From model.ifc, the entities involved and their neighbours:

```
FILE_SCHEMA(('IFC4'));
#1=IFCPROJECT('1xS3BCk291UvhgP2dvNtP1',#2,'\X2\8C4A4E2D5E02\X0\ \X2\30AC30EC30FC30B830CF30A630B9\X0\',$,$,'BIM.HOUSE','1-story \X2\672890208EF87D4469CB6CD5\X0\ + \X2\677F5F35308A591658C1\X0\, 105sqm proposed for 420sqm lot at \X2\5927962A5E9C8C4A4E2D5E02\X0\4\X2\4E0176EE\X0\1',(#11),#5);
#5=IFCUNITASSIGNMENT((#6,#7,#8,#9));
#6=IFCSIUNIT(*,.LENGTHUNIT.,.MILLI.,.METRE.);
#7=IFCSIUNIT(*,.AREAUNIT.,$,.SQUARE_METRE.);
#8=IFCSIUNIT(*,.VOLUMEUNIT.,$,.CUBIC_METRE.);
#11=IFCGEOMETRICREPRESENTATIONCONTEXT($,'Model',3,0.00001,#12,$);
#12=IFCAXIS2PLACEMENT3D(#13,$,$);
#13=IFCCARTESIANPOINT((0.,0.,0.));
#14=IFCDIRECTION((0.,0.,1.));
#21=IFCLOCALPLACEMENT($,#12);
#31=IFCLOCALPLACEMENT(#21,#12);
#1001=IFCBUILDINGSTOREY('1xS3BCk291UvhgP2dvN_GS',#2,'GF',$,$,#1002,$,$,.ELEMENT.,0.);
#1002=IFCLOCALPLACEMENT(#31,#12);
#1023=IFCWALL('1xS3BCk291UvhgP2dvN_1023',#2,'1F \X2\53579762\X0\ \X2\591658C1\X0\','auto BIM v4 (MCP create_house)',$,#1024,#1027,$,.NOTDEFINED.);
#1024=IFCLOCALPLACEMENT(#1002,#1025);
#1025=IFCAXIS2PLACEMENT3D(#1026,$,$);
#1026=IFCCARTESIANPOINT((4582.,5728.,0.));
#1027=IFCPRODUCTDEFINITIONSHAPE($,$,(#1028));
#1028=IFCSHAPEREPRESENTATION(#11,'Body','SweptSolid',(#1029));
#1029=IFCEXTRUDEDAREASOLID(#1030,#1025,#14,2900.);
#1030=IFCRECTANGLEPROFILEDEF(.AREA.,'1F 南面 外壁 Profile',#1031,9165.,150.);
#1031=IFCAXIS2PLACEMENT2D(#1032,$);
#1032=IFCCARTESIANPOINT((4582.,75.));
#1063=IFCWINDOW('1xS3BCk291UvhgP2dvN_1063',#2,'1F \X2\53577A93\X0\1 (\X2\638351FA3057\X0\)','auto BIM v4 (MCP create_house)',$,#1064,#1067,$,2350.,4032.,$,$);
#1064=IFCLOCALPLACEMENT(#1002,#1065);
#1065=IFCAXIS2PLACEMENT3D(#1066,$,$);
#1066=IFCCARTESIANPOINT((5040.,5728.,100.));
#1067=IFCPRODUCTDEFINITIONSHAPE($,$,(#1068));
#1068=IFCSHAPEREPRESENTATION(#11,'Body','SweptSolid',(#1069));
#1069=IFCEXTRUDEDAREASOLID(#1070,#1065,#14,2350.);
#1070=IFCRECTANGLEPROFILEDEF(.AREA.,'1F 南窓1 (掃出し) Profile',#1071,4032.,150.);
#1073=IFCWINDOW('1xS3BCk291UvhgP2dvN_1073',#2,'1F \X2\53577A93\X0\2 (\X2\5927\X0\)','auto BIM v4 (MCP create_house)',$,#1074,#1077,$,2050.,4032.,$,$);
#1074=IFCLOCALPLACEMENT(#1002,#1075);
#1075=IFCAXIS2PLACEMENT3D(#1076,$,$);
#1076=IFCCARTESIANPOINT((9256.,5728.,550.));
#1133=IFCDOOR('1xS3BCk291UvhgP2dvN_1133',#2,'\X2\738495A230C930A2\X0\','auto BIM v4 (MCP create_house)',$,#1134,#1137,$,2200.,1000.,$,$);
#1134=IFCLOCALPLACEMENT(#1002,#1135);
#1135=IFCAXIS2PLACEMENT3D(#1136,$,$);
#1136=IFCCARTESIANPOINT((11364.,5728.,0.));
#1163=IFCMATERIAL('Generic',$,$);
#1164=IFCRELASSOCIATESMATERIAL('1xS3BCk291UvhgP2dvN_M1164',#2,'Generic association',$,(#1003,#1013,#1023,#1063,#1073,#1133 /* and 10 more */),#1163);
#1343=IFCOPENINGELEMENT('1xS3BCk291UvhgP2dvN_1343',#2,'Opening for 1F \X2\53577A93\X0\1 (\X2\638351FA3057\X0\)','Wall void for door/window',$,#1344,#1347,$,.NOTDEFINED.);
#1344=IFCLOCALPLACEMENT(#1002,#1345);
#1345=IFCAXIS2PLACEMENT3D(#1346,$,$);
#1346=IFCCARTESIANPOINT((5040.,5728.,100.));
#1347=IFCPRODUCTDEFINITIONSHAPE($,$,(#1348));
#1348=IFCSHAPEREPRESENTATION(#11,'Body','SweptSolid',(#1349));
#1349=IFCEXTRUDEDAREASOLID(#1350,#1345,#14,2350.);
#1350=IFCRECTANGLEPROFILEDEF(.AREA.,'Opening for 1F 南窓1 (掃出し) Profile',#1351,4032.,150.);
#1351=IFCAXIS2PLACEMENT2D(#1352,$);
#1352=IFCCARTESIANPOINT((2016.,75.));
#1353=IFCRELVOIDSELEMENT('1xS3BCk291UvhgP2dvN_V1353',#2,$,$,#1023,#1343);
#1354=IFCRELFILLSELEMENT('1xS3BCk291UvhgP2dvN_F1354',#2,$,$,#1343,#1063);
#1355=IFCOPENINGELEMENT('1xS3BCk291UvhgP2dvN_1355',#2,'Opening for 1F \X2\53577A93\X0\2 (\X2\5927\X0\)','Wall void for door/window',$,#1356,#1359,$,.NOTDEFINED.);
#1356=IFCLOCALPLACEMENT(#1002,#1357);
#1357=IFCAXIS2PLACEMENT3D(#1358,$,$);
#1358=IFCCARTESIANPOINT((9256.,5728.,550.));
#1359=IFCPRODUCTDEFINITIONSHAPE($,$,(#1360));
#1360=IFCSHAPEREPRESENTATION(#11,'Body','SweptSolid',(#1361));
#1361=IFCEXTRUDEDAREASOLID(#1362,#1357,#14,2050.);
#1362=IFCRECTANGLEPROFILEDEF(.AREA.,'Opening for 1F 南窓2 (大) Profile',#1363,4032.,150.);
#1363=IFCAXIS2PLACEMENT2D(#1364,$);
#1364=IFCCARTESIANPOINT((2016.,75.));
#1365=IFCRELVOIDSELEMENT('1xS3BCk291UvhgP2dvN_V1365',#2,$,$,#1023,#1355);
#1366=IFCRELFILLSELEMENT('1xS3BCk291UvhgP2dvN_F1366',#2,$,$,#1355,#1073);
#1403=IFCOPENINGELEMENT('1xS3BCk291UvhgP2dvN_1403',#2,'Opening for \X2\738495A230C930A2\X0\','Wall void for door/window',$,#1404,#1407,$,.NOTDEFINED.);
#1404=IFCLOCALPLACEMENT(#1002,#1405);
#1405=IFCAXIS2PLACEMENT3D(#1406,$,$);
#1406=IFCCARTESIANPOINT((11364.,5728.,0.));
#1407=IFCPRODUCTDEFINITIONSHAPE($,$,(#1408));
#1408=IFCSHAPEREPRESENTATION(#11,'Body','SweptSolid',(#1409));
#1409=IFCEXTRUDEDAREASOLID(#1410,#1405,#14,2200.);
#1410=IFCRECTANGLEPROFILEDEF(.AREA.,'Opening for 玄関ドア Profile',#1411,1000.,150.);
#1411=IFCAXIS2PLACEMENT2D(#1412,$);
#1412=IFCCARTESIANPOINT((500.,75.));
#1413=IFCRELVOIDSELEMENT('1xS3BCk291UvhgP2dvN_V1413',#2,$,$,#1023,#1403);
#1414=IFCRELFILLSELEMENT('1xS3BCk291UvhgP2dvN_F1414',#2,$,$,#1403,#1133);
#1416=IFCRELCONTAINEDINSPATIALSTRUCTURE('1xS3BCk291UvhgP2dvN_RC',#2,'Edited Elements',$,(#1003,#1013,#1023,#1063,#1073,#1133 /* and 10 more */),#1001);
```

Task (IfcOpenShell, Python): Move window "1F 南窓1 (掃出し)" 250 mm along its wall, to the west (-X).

```python
import ifcopenshell
import ifcopenshell.api.geometry
import ifcopenshell.util.placement

model = ifcopenshell.open("model.ifc")

window = model.by_id(1063)
opening = window.FillsVoids[0].RelatingOpeningElement
wall = opening.VoidsElements[0].RelatingBuildingElement

wall_matrix = ifcopenshell.util.placement.get_local_placement(wall.ObjectPlacement)
shift = wall_matrix[:3, 0] * -250.0
before = ifcopenshell.util.placement.get_local_placement(window.ObjectPlacement)[:3, 3].copy()

# The window is not placed relative to its opening, so move both.
for product in (opening, window):
    matrix = ifcopenshell.util.placement.get_local_placement(product.ObjectPlacement)
    matrix[:3, 3] += shift
    ifcopenshell.api.geometry.edit_object_placement(model, product=product, matrix=matrix, is_si=False)

after = ifcopenshell.util.placement.get_local_placement(window.ObjectPlacement)[:3, 3]
print("window moved by", (after - before).round(3) + 0.0)

model.write("model_updated.ifc")
```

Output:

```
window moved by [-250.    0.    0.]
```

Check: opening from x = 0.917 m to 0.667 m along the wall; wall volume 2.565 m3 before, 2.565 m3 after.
